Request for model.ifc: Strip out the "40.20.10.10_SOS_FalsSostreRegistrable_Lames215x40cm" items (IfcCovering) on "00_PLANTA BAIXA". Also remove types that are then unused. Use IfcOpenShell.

First a look at what the model holds.

```python
import ifcopenshell
import ifcopenshell.util.element

model = ifcopenshell.open("model.ifc")
print(model.schema)
storey = next(s for s in model.by_type("IfcBuildingStorey") if s.Name == "00_PLANTA BAIXA")
coverings = [e for e in ifcopenshell.util.element.get_decomposition(storey) if e.is_a("IfcCovering")]
seen = {}
for e in coverings:
    element_type = ifcopenshell.util.element.get_type(e)
    name = element_type.Name if element_type not in (None, e) else None
    seen[name] = seen.get(name, 0) + 1
for name, count in sorted(seen.items(), key=str):
    print(count, "x", name)
```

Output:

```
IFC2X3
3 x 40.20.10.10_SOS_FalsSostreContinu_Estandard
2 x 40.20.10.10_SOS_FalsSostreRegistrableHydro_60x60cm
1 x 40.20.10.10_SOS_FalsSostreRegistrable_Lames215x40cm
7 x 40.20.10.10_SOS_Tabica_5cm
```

```python
import ifcopenshell
import ifcopenshell.api.root
import ifcopenshell.util.element

model = ifcopenshell.open("model.ifc")

storey = next(s for s in model.by_type("IfcBuildingStorey") if s.Name == "00_PLANTA BAIXA")
coverings = [e for e in ifcopenshell.util.element.get_decomposition(storey) if e.is_a("IfcCovering")]
targets = [e for e in coverings if (t := ifcopenshell.util.element.get_type(e)) not in (None, e) and t.Name == "40.20.10.10_SOS_FalsSostreRegistrable_Lames215x40cm"]
types = {ifcopenshell.util.element.get_type(e) for e in targets} - {None, *targets}

for e in targets:
    ifcopenshell.api.root.remove_product(model, product=e)
print(len(targets), "removed")

unused = [t for t in types if not ifcopenshell.util.element.get_types(t)]
for t in unused:
    ifcopenshell.api.root.remove_product(model, product=t)
print(len(unused), "unused types removed")

model.write("model_v2.ifc")
```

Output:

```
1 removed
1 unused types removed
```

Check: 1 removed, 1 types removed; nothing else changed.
